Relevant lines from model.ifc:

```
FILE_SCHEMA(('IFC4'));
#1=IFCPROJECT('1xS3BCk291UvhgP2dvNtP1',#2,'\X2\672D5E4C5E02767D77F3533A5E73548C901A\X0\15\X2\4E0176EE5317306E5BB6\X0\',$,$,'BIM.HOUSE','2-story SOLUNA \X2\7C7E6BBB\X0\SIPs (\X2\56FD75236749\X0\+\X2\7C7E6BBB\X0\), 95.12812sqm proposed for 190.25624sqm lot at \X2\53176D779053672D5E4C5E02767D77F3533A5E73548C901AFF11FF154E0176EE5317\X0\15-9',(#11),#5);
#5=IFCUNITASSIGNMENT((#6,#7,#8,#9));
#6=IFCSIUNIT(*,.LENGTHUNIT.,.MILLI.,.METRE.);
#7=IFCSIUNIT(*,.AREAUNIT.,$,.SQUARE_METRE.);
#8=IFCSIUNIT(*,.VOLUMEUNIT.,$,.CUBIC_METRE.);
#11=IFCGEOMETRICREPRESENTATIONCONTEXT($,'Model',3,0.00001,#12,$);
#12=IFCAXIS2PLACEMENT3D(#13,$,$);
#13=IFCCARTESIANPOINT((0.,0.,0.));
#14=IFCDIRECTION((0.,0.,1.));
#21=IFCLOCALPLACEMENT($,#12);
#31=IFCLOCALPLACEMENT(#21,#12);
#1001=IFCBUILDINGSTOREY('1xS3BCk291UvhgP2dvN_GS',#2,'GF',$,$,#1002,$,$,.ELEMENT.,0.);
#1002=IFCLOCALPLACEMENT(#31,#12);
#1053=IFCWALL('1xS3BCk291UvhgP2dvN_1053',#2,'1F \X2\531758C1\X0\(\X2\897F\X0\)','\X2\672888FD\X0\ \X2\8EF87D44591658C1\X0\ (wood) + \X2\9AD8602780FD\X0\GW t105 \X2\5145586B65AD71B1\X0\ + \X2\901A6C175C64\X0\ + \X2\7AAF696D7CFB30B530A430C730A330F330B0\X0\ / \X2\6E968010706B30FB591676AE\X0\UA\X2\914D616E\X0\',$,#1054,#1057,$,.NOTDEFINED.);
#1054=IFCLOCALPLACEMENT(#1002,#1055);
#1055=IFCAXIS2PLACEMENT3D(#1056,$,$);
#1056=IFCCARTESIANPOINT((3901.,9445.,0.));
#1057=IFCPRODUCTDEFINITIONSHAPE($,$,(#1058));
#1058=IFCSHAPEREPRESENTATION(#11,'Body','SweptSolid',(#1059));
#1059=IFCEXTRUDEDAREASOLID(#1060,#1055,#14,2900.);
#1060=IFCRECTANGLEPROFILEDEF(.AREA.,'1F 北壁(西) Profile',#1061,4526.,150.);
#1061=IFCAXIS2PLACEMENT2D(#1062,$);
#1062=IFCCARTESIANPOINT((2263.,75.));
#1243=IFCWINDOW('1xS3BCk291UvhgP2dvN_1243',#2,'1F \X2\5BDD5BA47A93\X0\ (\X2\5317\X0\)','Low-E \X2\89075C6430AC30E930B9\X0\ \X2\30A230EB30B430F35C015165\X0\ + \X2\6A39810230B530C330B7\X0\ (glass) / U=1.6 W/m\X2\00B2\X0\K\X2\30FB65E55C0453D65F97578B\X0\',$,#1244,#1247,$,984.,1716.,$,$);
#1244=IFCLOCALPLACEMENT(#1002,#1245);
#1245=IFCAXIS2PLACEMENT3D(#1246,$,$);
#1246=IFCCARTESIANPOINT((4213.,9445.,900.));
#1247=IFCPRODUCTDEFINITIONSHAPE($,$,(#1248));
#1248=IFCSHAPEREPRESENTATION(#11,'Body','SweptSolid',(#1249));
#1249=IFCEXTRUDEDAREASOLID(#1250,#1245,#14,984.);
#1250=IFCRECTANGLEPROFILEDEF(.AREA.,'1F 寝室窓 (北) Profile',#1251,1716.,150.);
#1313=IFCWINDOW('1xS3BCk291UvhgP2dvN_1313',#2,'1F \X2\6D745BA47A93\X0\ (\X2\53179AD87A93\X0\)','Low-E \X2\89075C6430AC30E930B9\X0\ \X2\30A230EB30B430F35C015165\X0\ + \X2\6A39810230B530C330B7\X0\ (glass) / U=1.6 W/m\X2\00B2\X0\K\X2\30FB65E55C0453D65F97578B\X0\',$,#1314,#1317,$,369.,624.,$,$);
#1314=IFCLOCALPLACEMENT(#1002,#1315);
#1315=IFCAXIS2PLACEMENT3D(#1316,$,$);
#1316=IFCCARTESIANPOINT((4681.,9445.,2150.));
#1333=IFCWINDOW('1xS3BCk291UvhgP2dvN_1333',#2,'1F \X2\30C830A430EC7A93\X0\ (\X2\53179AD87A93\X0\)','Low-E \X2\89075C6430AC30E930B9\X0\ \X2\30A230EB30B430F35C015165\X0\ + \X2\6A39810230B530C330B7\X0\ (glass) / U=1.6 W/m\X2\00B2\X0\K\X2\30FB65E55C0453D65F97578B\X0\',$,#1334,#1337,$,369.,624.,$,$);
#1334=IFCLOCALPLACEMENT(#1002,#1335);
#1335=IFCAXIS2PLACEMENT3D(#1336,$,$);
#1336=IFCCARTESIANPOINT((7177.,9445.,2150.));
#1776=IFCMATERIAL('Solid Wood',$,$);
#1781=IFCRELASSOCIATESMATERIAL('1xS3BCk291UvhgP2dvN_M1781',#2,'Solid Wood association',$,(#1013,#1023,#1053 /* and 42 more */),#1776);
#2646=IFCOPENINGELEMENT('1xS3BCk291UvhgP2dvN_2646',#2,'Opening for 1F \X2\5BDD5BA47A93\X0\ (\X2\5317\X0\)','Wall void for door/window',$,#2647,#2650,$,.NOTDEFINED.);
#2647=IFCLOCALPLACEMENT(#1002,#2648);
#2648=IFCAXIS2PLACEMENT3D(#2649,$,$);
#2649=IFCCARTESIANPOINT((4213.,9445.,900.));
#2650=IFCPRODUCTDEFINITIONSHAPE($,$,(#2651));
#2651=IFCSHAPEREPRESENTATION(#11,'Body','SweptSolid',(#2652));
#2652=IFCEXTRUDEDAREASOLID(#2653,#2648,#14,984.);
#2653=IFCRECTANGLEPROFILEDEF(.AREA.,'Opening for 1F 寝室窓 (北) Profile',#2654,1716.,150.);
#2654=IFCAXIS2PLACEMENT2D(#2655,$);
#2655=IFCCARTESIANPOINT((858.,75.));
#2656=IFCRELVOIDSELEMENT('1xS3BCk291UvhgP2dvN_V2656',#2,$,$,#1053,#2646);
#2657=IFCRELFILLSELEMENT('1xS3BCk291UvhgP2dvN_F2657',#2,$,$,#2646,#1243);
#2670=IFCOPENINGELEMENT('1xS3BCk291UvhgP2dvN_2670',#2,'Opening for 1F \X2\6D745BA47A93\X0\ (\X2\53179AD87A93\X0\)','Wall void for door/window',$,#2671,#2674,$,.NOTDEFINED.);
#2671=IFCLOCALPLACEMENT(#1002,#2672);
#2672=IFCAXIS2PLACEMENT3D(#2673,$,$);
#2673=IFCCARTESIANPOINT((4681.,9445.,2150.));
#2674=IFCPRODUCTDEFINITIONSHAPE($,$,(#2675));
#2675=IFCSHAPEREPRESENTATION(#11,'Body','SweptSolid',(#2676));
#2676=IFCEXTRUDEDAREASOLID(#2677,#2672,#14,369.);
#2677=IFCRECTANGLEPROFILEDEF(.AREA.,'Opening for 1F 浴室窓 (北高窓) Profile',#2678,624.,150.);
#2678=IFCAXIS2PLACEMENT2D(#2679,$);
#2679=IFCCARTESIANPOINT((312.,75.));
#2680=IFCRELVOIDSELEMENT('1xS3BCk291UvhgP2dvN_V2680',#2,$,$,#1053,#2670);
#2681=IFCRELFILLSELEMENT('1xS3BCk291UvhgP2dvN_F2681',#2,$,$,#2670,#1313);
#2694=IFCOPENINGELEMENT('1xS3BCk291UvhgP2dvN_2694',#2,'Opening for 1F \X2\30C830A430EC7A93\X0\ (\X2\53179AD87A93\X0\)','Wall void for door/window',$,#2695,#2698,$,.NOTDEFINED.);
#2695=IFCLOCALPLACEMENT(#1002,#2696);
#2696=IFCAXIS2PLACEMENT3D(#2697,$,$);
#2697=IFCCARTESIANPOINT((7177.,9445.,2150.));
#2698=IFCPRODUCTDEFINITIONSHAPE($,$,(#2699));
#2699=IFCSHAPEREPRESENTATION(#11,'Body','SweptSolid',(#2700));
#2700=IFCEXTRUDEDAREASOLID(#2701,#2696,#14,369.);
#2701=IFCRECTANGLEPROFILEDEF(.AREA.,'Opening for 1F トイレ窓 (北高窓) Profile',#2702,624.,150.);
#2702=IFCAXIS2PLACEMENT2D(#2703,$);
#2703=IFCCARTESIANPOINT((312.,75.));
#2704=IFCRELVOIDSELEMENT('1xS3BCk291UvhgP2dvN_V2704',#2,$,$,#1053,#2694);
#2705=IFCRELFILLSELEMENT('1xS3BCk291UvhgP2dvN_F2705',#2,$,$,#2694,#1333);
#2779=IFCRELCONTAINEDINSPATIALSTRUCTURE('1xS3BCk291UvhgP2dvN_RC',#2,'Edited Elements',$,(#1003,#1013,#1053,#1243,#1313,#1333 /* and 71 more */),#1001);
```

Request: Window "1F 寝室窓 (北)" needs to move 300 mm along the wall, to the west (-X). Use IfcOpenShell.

```python
import ifcopenshell
import ifcopenshell.api.geometry
import ifcopenshell.util.placement
import ifcopenshell.util.unit

model = ifcopenshell.open("model.ifc")
unit_scale = ifcopenshell.util.unit.calculate_unit_scale(model)

window = model.by_guid("1xS3BCk291UvhgP2dvN_1243")
opening = window.FillsVoids[0].RelatingOpeningElement
wall = opening.VoidsElements[0].RelatingBuildingElement

wall_matrix = ifcopenshell.util.placement.get_local_placement(wall.ObjectPlacement)
shift = wall_matrix[:3, 0] * -0.3 / unit_scale
before = ifcopenshell.util.placement.get_local_placement(window.ObjectPlacement)[:3, 3].copy()

# The window is not placed relative to its opening, so move both.
for product in (opening, window):
    matrix = ifcopenshell.util.placement.get_local_placement(product.ObjectPlacement)
    matrix[:3, 3] += shift
    ifcopenshell.api.geometry.edit_object_placement(model, product=product, matrix=matrix, is_si=False)

after = ifcopenshell.util.placement.get_local_placement(window.ObjectPlacement)[:3, 3]
print("window moved by", (after - before).round(3) + 0.0)

model.write("model-out.ifc")
```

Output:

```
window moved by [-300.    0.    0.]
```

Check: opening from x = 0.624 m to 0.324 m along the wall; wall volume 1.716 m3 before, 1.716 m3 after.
